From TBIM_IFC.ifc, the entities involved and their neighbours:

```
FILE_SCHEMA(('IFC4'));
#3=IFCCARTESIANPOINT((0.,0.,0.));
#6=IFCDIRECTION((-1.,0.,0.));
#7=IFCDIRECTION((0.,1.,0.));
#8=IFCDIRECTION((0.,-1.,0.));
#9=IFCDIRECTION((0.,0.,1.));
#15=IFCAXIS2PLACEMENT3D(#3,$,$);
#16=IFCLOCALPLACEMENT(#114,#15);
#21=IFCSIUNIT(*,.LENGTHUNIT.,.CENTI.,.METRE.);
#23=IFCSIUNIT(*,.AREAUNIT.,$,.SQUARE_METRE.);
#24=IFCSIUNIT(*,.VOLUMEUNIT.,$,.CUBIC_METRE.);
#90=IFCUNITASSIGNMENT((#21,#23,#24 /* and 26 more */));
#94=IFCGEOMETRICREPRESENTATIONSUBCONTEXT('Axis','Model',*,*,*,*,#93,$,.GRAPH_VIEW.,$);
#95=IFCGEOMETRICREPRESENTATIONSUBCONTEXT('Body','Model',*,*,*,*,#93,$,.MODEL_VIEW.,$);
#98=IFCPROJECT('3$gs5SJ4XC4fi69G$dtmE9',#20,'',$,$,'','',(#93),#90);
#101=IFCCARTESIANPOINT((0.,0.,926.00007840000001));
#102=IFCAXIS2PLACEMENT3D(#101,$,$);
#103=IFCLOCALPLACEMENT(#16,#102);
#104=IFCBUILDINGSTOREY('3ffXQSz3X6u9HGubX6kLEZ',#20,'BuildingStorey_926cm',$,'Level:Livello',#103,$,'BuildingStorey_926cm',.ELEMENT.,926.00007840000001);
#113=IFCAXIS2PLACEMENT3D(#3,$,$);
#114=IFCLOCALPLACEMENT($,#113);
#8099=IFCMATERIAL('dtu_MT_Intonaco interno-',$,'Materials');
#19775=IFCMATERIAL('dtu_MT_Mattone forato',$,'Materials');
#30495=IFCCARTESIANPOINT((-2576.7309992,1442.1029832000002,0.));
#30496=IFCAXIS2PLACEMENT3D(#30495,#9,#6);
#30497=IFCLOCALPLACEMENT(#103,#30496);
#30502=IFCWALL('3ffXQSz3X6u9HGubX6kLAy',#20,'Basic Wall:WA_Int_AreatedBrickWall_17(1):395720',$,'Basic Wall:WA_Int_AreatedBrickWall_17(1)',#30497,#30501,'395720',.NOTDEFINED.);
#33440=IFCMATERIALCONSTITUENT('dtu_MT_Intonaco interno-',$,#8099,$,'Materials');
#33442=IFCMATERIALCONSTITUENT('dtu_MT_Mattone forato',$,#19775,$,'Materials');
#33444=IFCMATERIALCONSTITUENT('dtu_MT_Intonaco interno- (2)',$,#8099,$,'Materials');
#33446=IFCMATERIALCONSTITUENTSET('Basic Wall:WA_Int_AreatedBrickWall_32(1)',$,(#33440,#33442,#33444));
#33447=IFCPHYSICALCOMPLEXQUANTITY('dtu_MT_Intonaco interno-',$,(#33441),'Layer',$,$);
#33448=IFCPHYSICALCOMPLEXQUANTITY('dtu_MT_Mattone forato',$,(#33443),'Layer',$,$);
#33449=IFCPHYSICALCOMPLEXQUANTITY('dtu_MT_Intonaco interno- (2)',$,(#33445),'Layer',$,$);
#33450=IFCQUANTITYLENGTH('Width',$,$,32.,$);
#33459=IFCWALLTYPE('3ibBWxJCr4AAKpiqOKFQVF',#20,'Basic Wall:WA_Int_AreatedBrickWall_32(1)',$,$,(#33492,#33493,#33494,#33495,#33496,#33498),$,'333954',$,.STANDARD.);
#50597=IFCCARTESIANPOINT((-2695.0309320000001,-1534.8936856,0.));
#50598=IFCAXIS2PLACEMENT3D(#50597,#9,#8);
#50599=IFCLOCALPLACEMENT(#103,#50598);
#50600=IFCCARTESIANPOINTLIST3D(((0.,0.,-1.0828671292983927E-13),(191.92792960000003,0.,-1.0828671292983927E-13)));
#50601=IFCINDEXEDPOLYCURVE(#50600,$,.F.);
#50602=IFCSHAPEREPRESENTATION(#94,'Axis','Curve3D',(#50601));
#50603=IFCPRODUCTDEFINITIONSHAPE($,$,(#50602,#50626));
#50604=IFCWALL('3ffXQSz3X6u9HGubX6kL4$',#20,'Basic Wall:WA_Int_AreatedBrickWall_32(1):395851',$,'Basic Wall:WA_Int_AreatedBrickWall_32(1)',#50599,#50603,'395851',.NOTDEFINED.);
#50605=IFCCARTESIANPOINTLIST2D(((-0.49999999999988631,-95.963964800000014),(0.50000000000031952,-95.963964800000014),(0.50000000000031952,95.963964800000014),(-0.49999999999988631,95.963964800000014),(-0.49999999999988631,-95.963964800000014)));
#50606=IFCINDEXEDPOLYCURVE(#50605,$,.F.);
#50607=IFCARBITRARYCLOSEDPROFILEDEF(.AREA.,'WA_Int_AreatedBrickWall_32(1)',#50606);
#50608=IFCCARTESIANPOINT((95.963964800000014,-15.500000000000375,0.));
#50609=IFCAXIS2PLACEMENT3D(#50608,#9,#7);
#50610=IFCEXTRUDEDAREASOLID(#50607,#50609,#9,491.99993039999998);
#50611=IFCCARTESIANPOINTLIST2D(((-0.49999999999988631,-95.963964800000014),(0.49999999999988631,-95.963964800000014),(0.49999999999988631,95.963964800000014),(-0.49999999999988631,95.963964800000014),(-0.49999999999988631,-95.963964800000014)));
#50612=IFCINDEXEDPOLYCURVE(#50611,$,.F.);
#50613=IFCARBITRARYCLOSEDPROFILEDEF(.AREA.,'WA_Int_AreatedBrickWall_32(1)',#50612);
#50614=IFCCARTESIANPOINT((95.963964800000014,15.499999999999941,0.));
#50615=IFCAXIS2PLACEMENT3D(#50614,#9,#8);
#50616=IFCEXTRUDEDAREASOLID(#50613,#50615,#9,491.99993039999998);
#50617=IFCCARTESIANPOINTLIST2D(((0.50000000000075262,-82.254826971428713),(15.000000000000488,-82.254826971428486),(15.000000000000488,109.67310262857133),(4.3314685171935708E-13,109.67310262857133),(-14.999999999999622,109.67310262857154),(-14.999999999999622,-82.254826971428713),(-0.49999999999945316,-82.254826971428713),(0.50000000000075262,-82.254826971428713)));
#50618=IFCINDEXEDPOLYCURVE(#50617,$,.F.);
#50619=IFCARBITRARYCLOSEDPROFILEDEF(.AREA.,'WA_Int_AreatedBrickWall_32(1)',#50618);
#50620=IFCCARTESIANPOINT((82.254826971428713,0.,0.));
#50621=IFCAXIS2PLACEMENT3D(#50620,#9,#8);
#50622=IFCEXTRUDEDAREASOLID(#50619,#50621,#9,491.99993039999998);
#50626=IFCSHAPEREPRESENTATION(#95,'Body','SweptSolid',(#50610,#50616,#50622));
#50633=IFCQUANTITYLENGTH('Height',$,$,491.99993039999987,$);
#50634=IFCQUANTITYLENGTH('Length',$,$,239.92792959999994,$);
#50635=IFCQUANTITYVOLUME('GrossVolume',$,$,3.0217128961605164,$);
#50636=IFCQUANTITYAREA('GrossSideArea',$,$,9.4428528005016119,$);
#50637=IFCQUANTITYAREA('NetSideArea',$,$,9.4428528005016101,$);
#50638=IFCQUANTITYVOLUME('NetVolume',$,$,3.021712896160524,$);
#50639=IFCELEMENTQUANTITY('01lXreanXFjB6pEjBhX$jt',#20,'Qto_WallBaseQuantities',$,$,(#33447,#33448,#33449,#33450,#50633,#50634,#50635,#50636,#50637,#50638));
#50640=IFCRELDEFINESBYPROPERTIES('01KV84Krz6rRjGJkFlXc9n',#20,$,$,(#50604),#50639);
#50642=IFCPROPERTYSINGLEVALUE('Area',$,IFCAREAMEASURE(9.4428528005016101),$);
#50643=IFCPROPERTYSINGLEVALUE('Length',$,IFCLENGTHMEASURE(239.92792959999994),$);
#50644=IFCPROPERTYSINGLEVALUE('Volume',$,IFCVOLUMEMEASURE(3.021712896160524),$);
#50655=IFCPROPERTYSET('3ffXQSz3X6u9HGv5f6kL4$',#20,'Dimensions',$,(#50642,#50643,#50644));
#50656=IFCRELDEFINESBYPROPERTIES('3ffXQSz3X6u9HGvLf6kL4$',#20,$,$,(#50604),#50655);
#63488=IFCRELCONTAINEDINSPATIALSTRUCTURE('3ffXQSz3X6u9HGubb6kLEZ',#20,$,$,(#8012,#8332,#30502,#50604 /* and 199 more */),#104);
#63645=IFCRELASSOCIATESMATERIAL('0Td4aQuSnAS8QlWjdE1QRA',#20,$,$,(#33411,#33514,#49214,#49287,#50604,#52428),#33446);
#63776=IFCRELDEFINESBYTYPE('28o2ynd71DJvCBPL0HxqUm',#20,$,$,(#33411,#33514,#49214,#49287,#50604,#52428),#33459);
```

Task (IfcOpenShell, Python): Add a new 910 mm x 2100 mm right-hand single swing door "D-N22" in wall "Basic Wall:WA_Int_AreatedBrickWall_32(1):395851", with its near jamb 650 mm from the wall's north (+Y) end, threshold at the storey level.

```python
import numpy as np
import ifcopenshell
import ifcopenshell.api.feature
import ifcopenshell.api.geometry
import ifcopenshell.api.pset
import ifcopenshell.api.root
import ifcopenshell.api.spatial
import ifcopenshell.geom
import ifcopenshell.util.element
import ifcopenshell.util.placement
import ifcopenshell.util.representation
import ifcopenshell.util.shape
import ifcopenshell.util.unit

model = ifcopenshell.open("TBIM_IFC.ifc")
unit_scale = ifcopenshell.util.unit.calculate_unit_scale(model)
area_scale = ifcopenshell.util.unit.calculate_unit_scale(model, "AREAUNIT")
volume_scale = ifcopenshell.util.unit.calculate_unit_scale(model, "VOLUMEUNIT")
settings = ifcopenshell.geom.settings()


def volume(element):
    """Net volume in cubic metres, openings subtracted."""
    shape = ifcopenshell.geom.create_shape(settings, element)
    return ifcopenshell.util.shape.get_volume(shape.geometry)


wall = model.by_guid("3ffXQSz3X6u9HGubX6kL4$")
storey = ifcopenshell.util.element.get_container(wall, ifc_class="IfcBuildingStorey")
context = ifcopenshell.util.representation.get_context(model, "Model", "Body", "MODEL_VIEW")
before = volume(wall)

width, height, from_end, sill = 0.91, 2.1, 0.65, 0.0  # metres

# The wall runs along its own X axis, and the end named is its -X end.
wall_shape = ifcopenshell.geom.create_shape(settings, wall)
x, y, z = ifcopenshell.util.shape.get_vertices(wall_shape.geometry).T
start = x.min() + from_end
face, thickness = float(y.min()), float(y.max() - y.min())
wall_matrix = ifcopenshell.util.placement.get_local_placement(wall.ObjectPlacement)
level = ifcopenshell.util.placement.get_local_placement(storey.ObjectPlacement)[2, 3]


def in_wall(x, y):
    """Placement at x, y metres in the wall's axes, at sill height."""
    matrix = wall_matrix.copy()
    matrix[:, 3] = wall_matrix @ np.array([x / unit_scale, y / unit_scale, 0.0, 1.0])
    matrix[2, 3] = level + sill / unit_scale
    return matrix


# Opening: a box that overshoots both wall faces by 50 mm.
opening = ifcopenshell.api.root.create_entity(model, ifc_class="IfcOpeningElement", predefined_type="OPENING")
box = ifcopenshell.api.geometry.add_wall_representation(
    model, context=context, length=width, height=height, thickness=thickness + 0.1
)
ifcopenshell.api.geometry.assign_representation(model, product=opening, representation=box)
ifcopenshell.api.geometry.edit_object_placement(model, product=opening, matrix=in_wall(start, face - 0.05), is_si=False)
ifcopenshell.api.feature.add_feature(model, feature=opening, element=wall)

door = ifcopenshell.api.root.create_entity(model, ifc_class="IfcDoor", name="D-N22", predefined_type="DOOR")
door.OverallWidth, door.OverallHeight = width / unit_scale, height / unit_scale
door.OperationType = "SINGLE_SWING_RIGHT"
body = ifcopenshell.api.geometry.add_door_representation(
    model,
    context=context,
    overall_width=door.OverallWidth,
    overall_height=door.OverallHeight,
    operation_type="SINGLE_SWING_RIGHT",
    lining_properties={"LiningDepth": thickness / unit_scale, "ThresholdDepth": thickness / unit_scale},
)
ifcopenshell.api.geometry.assign_representation(model, product=door, representation=body)
ifcopenshell.api.spatial.assign_container(model, products=[door], relating_structure=storey)
ifcopenshell.api.feature.add_filling(model, opening=opening, element=door)

# The lining spans the wall, so the door starts at the wall face.
ifcopenshell.api.geometry.edit_object_placement(model, product=door, matrix=in_wall(start, face), is_si=False)

after = volume(wall)

# Update the wall's stored quantities.
qto = model.by_id(ifcopenshell.util.element.get_pset(wall, "Qto_WallBaseQuantities", should_inherit=False)["id"])
ifcopenshell.api.pset.edit_qto(model, qto=qto, properties={
    "NetSideArea": after / thickness / area_scale,
    "NetVolume": after / volume_scale,
})
pset = model.by_id(ifcopenshell.util.element.get_pset(wall, "Dimensions", should_inherit=False)["id"])
ifcopenshell.api.pset.edit_pset(model, pset=pset, properties={
    "Area": model.create_entity("IfcAreaMeasure", after / thickness / area_scale),
    "Volume": model.create_entity("IfcVolumeMeasure", after / volume_scale),
})

print(f"wall volume {before:.3f} -> {after:.3f} m3")

model.write("TBIM_IFC_v2.ifc")
```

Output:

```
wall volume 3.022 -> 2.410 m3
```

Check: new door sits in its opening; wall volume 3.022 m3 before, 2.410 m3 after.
